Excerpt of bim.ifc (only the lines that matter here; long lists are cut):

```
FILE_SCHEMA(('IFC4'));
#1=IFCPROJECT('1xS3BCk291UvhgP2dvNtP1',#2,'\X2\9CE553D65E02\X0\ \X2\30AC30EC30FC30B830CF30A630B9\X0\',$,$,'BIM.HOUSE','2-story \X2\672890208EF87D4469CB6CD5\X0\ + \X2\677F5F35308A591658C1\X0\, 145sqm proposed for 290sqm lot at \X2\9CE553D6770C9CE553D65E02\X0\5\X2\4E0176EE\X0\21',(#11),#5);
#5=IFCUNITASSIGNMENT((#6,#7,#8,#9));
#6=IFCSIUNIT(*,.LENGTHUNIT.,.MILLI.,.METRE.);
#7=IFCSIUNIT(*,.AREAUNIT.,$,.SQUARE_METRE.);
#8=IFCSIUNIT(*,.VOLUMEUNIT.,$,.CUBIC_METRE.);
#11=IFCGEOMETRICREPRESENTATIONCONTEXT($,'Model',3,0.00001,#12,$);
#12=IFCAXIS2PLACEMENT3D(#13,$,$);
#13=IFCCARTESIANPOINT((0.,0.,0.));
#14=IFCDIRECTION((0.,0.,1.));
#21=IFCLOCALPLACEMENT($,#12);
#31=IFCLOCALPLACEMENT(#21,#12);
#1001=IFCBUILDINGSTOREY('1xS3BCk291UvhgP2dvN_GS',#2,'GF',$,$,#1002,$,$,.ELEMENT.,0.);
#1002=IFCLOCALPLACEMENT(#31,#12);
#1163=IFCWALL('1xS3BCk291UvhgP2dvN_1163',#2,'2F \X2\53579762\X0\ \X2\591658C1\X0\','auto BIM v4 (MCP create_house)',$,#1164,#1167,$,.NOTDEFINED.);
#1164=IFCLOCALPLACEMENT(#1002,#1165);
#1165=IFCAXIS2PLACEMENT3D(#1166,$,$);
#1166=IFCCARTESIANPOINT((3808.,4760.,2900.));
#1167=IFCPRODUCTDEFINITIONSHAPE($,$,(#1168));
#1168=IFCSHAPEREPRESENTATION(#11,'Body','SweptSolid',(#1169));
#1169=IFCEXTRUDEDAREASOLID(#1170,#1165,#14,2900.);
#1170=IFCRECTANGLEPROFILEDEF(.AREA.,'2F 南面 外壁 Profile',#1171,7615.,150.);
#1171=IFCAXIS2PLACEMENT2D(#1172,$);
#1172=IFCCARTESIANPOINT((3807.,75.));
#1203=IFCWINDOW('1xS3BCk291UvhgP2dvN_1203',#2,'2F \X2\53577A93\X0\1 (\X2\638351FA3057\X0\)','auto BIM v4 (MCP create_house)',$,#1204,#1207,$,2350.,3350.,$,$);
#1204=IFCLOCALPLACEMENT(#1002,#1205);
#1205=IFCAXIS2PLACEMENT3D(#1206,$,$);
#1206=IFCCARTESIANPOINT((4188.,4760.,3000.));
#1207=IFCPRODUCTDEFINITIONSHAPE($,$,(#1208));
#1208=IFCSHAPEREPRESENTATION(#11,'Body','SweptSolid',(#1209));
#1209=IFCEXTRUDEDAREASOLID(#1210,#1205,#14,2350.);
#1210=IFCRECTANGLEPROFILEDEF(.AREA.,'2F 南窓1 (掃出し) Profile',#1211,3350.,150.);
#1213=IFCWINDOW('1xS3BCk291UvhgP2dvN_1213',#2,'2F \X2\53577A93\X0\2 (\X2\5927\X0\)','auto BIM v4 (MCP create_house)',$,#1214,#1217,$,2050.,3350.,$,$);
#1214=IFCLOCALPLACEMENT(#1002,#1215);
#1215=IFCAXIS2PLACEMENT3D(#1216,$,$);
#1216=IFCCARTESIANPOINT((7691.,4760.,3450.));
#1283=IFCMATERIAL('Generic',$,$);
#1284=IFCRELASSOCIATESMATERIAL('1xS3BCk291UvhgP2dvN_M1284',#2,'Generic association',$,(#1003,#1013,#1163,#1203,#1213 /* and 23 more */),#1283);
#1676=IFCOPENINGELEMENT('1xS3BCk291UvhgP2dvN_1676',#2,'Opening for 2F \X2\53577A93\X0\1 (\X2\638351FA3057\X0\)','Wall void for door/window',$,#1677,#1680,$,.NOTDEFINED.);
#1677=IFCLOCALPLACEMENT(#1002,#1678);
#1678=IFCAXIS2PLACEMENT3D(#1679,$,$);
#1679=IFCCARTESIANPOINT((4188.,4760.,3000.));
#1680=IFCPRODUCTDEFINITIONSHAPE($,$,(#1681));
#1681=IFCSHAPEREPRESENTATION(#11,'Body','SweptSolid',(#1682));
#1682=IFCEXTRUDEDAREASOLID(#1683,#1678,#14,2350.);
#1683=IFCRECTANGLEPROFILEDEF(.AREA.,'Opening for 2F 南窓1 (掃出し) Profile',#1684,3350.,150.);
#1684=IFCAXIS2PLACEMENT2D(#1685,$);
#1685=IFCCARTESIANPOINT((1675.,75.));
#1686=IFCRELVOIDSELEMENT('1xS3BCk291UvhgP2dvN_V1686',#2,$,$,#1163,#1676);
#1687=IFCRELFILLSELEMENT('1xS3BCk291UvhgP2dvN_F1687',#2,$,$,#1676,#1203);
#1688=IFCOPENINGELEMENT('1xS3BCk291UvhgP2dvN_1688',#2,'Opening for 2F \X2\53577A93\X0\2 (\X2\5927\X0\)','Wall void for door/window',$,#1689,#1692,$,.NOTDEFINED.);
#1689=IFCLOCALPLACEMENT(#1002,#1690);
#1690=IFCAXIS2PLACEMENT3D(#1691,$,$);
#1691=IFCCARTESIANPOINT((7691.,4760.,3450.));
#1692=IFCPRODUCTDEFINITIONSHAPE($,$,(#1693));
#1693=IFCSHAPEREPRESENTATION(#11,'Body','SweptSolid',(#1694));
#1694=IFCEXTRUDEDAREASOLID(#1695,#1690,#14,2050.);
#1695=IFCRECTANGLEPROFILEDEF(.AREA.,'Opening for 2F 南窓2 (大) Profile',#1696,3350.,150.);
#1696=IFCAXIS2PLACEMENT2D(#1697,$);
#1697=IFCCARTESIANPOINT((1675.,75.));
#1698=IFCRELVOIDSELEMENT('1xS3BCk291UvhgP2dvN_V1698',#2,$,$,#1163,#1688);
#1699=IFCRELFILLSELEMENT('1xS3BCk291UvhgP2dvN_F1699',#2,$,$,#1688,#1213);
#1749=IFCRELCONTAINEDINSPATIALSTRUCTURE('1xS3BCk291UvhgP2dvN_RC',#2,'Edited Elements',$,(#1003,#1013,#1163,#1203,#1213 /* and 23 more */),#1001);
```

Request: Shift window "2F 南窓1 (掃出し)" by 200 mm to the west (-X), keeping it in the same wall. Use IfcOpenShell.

```python
import ifcopenshell
import ifcopenshell.api.geometry
import ifcopenshell.util.placement
import ifcopenshell.util.unit

model = ifcopenshell.open("bim.ifc")
unit_scale = ifcopenshell.util.unit.calculate_unit_scale(model)

window = model.by_id(1203)
opening = window.FillsVoids[0].RelatingOpeningElement
wall = opening.VoidsElements[0].RelatingBuildingElement

wall_matrix = ifcopenshell.util.placement.get_local_placement(wall.ObjectPlacement)
shift = wall_matrix[:3, 0] * -0.2 / unit_scale
before = ifcopenshell.util.placement.get_local_placement(window.ObjectPlacement)[:3, 3].copy()

# The window is not placed relative to its opening, so move both.
for product in (opening, window):
    matrix = ifcopenshell.util.placement.get_local_placement(product.ObjectPlacement)
    matrix[:3, 3] += shift
    ifcopenshell.api.geometry.edit_object_placement(model, product=product, matrix=matrix, is_si=False)

after = ifcopenshell.util.placement.get_local_placement(window.ObjectPlacement)[:3, 3]
print("window moved by", (after - before).round(3) + 0.0)

model.write("bim_v2.ifc")
```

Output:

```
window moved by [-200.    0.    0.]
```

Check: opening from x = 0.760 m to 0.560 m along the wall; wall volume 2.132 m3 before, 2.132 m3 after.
